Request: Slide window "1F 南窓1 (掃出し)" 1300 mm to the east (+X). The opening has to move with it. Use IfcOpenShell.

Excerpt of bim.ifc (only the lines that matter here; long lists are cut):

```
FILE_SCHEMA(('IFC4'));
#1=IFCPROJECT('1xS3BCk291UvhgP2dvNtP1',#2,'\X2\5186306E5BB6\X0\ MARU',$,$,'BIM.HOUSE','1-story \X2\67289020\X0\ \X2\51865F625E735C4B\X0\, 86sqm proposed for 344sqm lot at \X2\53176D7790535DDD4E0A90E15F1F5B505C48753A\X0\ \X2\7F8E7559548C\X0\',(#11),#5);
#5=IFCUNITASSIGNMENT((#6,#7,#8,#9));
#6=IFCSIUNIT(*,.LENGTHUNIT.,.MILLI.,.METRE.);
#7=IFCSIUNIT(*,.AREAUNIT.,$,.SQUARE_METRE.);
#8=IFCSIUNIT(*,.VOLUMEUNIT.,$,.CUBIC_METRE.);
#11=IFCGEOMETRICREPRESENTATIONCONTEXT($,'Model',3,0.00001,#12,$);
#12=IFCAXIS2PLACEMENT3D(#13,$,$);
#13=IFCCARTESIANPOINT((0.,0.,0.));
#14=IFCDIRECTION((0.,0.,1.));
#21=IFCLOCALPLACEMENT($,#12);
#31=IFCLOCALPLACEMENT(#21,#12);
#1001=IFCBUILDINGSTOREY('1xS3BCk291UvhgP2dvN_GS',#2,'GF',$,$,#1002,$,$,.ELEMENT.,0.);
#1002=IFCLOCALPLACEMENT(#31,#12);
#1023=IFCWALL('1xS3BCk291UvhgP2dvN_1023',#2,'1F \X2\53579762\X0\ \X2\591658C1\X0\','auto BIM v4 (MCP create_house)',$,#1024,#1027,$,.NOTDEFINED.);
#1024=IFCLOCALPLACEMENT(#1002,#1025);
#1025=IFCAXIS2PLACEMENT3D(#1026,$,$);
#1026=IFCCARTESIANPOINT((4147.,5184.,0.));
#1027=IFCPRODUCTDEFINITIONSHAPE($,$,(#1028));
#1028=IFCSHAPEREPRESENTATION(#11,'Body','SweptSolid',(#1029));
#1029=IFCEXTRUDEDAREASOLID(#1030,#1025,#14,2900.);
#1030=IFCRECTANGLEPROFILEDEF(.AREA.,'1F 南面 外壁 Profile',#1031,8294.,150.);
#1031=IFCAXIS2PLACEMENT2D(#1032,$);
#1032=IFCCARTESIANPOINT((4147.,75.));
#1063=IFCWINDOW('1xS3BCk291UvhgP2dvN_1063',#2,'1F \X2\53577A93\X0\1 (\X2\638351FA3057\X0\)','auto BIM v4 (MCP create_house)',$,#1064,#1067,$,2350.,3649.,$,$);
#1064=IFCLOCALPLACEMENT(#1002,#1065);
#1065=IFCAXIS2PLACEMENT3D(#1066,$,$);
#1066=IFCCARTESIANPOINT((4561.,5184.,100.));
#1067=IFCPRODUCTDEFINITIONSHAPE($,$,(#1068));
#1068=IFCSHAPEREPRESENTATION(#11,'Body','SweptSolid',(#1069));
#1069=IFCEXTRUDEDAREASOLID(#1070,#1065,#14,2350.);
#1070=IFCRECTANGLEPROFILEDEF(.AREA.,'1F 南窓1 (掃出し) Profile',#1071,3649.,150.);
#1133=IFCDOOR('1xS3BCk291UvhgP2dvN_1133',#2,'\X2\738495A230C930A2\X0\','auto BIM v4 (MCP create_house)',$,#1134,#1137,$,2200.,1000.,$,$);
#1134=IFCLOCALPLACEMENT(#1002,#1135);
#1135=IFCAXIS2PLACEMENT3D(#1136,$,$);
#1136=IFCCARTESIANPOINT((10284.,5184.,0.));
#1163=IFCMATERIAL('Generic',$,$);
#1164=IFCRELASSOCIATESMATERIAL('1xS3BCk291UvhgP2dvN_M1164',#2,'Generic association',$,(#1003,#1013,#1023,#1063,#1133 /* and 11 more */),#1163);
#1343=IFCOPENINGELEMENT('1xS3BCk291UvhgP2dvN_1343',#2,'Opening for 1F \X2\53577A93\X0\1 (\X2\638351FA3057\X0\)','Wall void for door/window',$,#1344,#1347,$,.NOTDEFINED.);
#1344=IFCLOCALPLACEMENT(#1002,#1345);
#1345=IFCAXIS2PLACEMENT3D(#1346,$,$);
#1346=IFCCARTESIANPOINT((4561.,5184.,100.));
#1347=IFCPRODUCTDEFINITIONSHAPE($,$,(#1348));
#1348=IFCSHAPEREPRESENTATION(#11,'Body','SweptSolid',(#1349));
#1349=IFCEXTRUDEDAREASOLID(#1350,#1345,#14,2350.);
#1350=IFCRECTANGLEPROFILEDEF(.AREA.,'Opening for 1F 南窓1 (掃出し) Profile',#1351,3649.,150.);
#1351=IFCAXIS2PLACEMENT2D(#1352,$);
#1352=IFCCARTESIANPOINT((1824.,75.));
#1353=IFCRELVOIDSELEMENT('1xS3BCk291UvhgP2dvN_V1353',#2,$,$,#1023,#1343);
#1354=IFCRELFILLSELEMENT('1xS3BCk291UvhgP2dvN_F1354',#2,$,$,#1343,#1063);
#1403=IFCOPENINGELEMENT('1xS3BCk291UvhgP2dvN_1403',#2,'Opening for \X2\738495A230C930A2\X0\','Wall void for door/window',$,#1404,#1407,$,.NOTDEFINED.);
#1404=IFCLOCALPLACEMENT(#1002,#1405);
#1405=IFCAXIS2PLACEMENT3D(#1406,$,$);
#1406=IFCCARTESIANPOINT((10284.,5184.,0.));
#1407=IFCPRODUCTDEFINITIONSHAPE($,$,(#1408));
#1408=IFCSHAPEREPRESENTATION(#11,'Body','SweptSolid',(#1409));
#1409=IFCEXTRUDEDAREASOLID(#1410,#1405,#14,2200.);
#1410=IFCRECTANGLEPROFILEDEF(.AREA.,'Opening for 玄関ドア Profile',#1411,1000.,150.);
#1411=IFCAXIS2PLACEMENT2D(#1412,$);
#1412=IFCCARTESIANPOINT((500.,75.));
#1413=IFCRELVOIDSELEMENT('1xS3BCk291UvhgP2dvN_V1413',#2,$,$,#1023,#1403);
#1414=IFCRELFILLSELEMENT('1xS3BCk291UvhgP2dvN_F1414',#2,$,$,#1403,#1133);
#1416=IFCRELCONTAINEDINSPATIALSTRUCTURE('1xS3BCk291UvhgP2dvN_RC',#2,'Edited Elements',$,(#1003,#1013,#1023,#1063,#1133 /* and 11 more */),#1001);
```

```python
import ifcopenshell
import ifcopenshell.api.geometry
import ifcopenshell.util.placement
import ifcopenshell.util.unit

model = ifcopenshell.open("bim.ifc")
unit_scale = ifcopenshell.util.unit.calculate_unit_scale(model)

window = model.by_id(1063)
opening = window.FillsVoids[0].RelatingOpeningElement
wall = opening.VoidsElements[0].RelatingBuildingElement

wall_matrix = ifcopenshell.util.placement.get_local_placement(wall.ObjectPlacement)
shift = wall_matrix[:3, 0] * 1.3 / unit_scale
before = ifcopenshell.util.placement.get_local_placement(window.ObjectPlacement)[:3, 3].copy()

# The window is not placed relative to its opening, so move both.
for product in (opening, window):
    matrix = ifcopenshell.util.placement.get_local_placement(product.ObjectPlacement)
    matrix[:3, 3] += shift
    ifcopenshell.api.geometry.edit_object_placement(model, product=product, matrix=matrix, is_si=False)

after = ifcopenshell.util.placement.get_local_placement(window.ObjectPlacement)[:3, 3]
print("window moved by", (after - before).round(3) + 0.0)

model.write("bim_edited.ifc")
```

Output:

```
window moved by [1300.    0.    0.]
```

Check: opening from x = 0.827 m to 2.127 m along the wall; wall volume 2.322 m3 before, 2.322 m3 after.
